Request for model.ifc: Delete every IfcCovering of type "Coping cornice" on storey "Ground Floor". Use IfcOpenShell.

First a look at what the model holds.

```python
import ifcopenshell
import ifcopenshell.util.element

model = ifcopenshell.open("model.ifc")
print(model.schema)
storey = next(s for s in model.by_type("IfcBuildingStorey") if s.Name == "Ground Floor")
coverings = [e for e in ifcopenshell.util.element.get_decomposition(storey) if e.is_a("IfcCovering")]
seen = {}
for e in coverings:
    element_type = ifcopenshell.util.element.get_type(e)
    name = element_type.Name if element_type not in (None, e) else None
    seen[name] = seen.get(name, 0) + 1
for name, count in sorted(seen.items(), key=str):
    print(count, "x", name)
```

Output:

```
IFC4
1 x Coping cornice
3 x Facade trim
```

```python
import ifcopenshell
import ifcopenshell.api.root
import ifcopenshell.util.element

model = ifcopenshell.open("model.ifc")

storey = next(s for s in model.by_type("IfcBuildingStorey") if s.Name == "Ground Floor")
coverings = [e for e in ifcopenshell.util.element.get_decomposition(storey) if e.is_a("IfcCovering")]
targets = [e for e in coverings if (t := ifcopenshell.util.element.get_type(e)) not in (None, e) and t.Name == "Coping cornice"]

for e in targets:
    ifcopenshell.api.root.remove_product(model, product=e)
print(len(targets), "removed")

model.write("model-out.ifc")
```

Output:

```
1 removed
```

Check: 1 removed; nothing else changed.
